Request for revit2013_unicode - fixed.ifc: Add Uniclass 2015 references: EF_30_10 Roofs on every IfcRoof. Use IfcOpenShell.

First a look at what the model holds.

```python
import ifcopenshell

model = ifcopenshell.open("revit2013_unicode - fixed.ifc")
print(model.schema)
print("classifications:", [c.Name for c in model.by_type("IfcClassification")])
for ifc_class in ("IfcDoor", "IfcRoof", "IfcStair", "IfcWall", "IfcWindow"):
    print(ifc_class, len(model.by_type(ifc_class)))
```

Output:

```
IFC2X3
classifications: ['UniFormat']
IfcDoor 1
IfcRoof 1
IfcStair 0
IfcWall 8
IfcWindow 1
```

```python
import ifcopenshell
import ifcopenshell.api.classification

model = ifcopenshell.open("revit2013_unicode - fixed.ifc")

# IFC2X3 requires Source and Edition and has no link from the project to the system.
system = model.create_entity("IfcClassification", Source="NBS", Edition="2015", Name="Uniclass 2015")

codes = {
    "IfcRoof": ("EF_30_10", "Roofs"),
}
for ifc_class, (code, name) in codes.items():
    products = model.by_type(ifc_class)
    ifcopenshell.api.classification.add_reference(
        model, products=products, classification=system, identification=code, name=name
    )
    print(code, len(products))

model.write("revit2013_unicode - fixed_edited.ifc")
```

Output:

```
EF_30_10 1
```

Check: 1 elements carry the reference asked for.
